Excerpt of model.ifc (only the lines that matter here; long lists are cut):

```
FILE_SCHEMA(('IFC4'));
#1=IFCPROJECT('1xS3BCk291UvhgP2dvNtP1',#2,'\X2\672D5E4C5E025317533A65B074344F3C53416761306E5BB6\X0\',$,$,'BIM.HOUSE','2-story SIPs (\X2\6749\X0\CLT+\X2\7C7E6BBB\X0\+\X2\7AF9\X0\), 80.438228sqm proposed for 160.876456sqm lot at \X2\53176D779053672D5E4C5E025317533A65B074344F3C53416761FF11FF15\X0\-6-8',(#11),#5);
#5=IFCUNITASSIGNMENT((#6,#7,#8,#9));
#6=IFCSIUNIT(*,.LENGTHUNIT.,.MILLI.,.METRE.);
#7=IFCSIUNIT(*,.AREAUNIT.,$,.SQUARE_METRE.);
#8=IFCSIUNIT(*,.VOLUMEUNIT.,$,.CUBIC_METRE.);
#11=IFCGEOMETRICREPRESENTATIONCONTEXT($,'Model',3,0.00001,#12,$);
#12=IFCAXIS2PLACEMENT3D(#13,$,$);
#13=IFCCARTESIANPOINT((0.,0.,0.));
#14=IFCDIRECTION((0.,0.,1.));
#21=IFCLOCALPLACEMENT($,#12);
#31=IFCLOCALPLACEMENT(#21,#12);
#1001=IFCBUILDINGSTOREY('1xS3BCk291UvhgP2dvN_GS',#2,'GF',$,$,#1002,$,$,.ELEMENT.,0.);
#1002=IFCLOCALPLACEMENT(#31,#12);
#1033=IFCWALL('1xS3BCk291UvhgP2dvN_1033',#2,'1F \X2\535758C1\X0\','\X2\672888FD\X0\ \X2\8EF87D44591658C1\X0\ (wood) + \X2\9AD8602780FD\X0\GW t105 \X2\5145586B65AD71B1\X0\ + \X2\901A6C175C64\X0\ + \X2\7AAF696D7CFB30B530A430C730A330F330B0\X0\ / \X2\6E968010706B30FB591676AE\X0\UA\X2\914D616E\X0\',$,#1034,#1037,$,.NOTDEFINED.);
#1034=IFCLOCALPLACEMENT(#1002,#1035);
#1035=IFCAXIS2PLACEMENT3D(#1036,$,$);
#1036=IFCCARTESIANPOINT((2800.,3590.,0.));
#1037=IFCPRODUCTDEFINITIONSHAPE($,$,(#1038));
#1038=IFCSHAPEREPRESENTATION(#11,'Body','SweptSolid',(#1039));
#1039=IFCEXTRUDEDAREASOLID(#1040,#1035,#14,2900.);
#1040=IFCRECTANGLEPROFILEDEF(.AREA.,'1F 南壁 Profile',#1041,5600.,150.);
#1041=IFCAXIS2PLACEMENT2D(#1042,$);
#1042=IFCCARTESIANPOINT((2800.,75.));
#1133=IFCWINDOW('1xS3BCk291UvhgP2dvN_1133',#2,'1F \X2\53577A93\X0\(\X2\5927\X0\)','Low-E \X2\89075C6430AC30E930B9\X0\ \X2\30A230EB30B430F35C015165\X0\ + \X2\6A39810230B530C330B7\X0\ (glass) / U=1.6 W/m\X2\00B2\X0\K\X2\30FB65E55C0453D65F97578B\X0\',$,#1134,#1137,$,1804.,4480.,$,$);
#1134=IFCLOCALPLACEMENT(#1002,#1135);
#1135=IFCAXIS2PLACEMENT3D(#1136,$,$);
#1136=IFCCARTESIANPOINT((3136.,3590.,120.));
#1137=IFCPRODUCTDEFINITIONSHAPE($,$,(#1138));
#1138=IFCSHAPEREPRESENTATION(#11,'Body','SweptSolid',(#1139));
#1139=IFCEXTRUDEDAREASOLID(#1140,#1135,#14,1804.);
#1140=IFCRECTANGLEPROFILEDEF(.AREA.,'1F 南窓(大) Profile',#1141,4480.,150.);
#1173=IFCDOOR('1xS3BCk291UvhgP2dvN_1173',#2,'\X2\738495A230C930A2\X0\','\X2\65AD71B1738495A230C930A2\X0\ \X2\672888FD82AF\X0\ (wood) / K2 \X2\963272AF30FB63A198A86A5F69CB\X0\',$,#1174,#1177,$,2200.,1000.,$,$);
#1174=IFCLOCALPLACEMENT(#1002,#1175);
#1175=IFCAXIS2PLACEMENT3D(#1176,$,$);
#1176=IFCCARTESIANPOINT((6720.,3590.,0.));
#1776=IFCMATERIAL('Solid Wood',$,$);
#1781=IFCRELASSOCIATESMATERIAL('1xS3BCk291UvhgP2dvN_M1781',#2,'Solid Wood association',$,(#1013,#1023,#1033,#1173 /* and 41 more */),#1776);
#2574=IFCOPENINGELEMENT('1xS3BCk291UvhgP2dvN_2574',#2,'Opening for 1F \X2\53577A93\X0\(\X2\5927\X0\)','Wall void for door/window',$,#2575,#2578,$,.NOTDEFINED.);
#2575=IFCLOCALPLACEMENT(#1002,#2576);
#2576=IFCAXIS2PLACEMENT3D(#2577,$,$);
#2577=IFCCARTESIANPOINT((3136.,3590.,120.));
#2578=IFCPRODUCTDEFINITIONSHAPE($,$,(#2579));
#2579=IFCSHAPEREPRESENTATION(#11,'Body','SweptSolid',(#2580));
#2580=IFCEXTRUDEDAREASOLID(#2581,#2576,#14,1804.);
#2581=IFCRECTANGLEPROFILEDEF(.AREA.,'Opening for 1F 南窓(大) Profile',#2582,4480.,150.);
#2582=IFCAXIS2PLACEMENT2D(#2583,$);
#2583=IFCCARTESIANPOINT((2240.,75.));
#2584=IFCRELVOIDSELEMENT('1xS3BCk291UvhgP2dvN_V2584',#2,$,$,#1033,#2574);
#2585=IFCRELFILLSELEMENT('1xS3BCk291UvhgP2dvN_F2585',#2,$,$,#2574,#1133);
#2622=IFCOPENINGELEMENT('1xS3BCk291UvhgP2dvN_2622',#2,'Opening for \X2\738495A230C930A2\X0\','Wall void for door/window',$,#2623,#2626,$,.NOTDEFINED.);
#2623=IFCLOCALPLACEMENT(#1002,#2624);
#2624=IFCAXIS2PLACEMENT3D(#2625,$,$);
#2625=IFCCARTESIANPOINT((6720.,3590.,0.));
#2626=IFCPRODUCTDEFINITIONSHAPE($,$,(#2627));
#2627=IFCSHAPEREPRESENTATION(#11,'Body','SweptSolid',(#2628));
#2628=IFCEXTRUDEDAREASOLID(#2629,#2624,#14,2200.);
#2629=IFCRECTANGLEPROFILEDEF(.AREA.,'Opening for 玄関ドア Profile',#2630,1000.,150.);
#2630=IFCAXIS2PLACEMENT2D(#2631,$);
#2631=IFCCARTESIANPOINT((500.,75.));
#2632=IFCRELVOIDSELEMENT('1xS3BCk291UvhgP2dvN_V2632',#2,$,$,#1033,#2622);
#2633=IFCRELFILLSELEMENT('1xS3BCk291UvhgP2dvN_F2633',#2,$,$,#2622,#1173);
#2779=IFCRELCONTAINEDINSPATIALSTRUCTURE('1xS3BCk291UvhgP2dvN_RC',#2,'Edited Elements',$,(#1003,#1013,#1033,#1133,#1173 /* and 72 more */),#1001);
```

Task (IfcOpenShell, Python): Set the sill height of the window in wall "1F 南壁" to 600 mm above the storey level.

```python
import numpy as np
import ifcopenshell
import ifcopenshell.api.geometry
import ifcopenshell.geom
import ifcopenshell.util.element
import ifcopenshell.util.placement
import ifcopenshell.util.shape
import ifcopenshell.util.unit

model = ifcopenshell.open("model.ifc")
unit_scale = ifcopenshell.util.unit.calculate_unit_scale(model)

window = model.by_guid("1xS3BCk291UvhgP2dvN_1133")
opening = window.FillsVoids[0].RelatingOpeningElement
storey = ifcopenshell.util.element.get_container(window, ifc_class="IfcBuildingStorey")
level = ifcopenshell.util.placement.get_local_placement(storey.ObjectPlacement)[2, 3]

# The opening's origin need not be at the sill, so measure its lowest point.
shape = ifcopenshell.geom.create_shape(ifcopenshell.geom.settings(), opening)
bottom = ifcopenshell.util.shape.get_shape_bottom_elevation(shape, shape.geometry) / unit_scale
dz = level + 600.0 - bottom

shift = np.array([0.0, 0.0, dz])
# The window is not placed relative to its opening, so move both.
for product in (opening, window):
    matrix = ifcopenshell.util.placement.get_local_placement(product.ObjectPlacement)
    matrix[:3, 3] += shift
    ifcopenshell.api.geometry.edit_object_placement(model, product=product, matrix=matrix, is_si=False)

print(f"moved by {dz * unit_scale:+.3f} m")

model.write("model_v2.ifc")
```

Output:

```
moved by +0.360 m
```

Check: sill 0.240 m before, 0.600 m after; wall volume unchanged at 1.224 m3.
